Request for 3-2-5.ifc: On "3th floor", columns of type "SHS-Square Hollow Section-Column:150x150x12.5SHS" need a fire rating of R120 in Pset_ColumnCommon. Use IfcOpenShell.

First a look at what the model holds.

```python
import ifcopenshell
import ifcopenshell.util.element

model = ifcopenshell.open("3-2-5.ifc")
print(model.schema)
storey = next(s for s in model.by_type("IfcBuildingStorey") if s.Name == "3th floor")
columns = [e for e in ifcopenshell.util.element.get_decomposition(storey) if e.is_a("IfcColumn")]
seen = {}
for e in columns:
    element_type = ifcopenshell.util.element.get_type(e)
    key = (element_type.Name if element_type != e and element_type else None, ifcopenshell.util.element.get_pset(e, "Pset_ColumnCommon", "FireRating"))
    seen[key] = seen.get(key, 0) + 1
for (name, value), count in sorted(seen.items(), key=str):
    print(count, "x", name, "|", value)
```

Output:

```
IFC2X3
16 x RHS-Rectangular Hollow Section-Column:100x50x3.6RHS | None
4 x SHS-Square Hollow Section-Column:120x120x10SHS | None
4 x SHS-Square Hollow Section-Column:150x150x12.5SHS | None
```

```python
import ifcopenshell
import ifcopenshell.api.pset
import ifcopenshell.util.element

model = ifcopenshell.open("3-2-5.ifc")

storey = next(s for s in model.by_type("IfcBuildingStorey") if s.Name == "3th floor")
columns = [e for e in ifcopenshell.util.element.get_decomposition(storey) if e.is_a("IfcColumn")]

count = 0
for e in columns:
    element_type = ifcopenshell.util.element.get_type(e)
    if element_type in (None, e) or element_type.Name != "SHS-Square Hollow Section-Column:150x150x12.5SHS":
        continue
    # add_pset returns the element's existing set when there is one.
    pset = ifcopenshell.api.pset.add_pset(model, product=e, name="Pset_ColumnCommon")
    ifcopenshell.api.pset.edit_pset(model, pset=pset, properties={"FireRating": "R120"})
    count += 1

print(count, "columns updated")

model.write("3-2-5-out.ifc")
```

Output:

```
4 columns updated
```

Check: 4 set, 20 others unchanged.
